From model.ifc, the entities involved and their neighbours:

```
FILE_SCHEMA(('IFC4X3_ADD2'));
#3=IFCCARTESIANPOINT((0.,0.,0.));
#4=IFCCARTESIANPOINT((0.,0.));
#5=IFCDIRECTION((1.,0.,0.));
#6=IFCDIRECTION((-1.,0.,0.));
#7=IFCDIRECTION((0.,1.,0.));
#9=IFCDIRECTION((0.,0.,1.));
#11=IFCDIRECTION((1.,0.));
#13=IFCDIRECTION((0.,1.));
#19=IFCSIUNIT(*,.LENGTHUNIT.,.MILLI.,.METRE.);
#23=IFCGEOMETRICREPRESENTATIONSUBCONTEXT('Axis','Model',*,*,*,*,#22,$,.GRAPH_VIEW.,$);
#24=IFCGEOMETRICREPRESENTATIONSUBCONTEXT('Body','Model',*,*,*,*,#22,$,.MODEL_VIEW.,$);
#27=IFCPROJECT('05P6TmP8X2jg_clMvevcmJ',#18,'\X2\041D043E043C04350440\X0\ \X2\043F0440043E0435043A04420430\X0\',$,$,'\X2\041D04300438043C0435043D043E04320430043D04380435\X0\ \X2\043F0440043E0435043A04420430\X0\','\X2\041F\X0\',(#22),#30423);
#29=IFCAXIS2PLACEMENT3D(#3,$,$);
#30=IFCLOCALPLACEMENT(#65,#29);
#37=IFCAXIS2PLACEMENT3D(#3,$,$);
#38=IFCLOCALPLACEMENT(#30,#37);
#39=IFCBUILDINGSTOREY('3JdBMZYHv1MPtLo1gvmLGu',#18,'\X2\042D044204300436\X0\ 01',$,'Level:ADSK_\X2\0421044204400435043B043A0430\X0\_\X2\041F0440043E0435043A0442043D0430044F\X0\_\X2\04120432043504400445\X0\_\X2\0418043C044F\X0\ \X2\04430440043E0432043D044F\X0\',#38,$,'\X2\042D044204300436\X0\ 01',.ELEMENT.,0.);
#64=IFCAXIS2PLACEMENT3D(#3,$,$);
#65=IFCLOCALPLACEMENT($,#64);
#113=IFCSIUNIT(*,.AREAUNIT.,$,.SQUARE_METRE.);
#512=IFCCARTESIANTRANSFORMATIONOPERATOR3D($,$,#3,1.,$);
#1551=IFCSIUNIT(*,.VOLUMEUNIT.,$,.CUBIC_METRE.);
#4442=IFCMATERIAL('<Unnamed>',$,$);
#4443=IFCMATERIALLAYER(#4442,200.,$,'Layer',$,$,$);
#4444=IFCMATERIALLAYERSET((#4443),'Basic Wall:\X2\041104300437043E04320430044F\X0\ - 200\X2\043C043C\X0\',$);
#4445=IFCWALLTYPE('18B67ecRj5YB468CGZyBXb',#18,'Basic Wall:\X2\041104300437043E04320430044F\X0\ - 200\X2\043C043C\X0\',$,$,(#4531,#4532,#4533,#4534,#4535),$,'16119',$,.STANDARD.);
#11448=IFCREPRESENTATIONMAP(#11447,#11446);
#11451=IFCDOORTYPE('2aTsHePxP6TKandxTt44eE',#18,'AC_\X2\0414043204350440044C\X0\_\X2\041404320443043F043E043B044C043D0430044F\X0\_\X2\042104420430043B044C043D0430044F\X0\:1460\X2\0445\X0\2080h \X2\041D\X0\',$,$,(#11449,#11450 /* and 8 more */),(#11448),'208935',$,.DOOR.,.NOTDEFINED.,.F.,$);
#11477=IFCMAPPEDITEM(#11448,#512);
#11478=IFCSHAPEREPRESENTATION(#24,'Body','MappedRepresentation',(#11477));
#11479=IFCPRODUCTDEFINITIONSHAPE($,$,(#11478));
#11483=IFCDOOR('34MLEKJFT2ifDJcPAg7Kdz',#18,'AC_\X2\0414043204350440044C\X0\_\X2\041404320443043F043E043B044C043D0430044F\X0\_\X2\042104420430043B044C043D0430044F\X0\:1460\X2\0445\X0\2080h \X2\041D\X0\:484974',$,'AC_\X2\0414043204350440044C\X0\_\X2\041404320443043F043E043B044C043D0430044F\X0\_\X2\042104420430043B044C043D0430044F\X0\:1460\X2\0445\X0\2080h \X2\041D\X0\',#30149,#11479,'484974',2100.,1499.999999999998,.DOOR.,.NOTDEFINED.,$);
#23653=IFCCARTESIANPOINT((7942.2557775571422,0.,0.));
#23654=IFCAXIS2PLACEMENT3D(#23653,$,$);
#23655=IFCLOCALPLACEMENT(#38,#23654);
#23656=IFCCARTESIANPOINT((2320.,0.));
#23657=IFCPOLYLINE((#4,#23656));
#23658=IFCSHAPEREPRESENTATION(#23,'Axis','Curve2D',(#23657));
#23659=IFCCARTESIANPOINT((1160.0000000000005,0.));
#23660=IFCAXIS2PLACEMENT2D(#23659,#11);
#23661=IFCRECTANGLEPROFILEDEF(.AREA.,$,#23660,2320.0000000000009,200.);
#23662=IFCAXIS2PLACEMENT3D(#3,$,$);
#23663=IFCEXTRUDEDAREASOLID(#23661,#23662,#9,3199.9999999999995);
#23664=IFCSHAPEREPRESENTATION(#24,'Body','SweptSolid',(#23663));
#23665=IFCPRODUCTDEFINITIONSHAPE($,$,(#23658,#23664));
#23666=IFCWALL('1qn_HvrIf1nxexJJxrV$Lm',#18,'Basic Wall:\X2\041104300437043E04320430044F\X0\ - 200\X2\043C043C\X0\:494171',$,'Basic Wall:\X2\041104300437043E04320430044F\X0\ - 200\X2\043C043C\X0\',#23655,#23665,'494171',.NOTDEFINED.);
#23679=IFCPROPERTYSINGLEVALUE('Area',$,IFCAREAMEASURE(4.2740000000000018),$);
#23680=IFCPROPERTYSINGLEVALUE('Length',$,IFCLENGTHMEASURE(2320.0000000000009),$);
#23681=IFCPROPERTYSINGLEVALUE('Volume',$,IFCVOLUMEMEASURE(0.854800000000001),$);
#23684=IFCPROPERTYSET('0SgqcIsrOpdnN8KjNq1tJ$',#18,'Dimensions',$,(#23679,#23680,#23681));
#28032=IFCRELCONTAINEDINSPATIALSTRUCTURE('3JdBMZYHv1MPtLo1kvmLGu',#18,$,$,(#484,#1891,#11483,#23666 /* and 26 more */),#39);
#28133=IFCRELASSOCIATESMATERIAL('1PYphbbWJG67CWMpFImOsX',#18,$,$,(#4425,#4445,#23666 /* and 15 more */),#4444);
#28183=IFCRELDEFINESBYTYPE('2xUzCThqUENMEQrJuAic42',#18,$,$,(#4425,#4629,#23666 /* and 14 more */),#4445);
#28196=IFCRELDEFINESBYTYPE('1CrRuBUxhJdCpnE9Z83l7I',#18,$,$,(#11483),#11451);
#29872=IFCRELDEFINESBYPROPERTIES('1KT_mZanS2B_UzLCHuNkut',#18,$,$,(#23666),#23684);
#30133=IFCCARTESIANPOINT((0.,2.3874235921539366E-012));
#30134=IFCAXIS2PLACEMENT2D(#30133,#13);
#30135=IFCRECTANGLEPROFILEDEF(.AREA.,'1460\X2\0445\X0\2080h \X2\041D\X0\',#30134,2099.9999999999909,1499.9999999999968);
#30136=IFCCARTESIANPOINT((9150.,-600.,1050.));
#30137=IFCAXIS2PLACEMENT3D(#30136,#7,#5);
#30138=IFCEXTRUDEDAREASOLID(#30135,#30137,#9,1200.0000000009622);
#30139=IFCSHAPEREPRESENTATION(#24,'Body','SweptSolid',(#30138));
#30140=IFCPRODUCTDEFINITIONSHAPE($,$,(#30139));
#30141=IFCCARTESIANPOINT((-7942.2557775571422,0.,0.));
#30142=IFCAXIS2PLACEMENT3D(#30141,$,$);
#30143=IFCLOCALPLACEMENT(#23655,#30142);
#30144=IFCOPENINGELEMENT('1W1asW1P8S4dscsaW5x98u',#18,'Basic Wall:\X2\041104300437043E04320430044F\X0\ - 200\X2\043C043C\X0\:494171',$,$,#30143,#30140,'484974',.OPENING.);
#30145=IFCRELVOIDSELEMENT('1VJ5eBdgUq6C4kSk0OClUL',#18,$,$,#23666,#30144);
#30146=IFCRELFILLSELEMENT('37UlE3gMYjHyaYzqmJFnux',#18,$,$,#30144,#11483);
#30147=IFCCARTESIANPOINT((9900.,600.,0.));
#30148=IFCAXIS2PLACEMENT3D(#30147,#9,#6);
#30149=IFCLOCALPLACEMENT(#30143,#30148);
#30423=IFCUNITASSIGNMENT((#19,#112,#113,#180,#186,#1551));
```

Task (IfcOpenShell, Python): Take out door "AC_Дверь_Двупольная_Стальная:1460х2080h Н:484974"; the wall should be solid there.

```python
import ifcopenshell
import ifcopenshell.api.feature
import ifcopenshell.api.pset
import ifcopenshell.api.root
import ifcopenshell.geom
import ifcopenshell.util.element
import ifcopenshell.util.shape
import ifcopenshell.util.unit

model = ifcopenshell.open("model.ifc")
area_scale = ifcopenshell.util.unit.calculate_unit_scale(model, "AREAUNIT")
volume_scale = ifcopenshell.util.unit.calculate_unit_scale(model, "VOLUMEUNIT")
settings = ifcopenshell.geom.settings()


def volume(element):
    """Net volume in cubic metres, openings subtracted."""
    shape = ifcopenshell.geom.create_shape(settings, element)
    return ifcopenshell.util.shape.get_volume(shape.geometry)


door = model.by_guid("34MLEKJFT2ifDJcPAg7Kdz")
opening = door.FillsVoids[0].RelatingOpeningElement
wall = opening.VoidsElements[0].RelatingBuildingElement
before = volume(wall)

ifcopenshell.api.root.remove_product(model, product=door)
ifcopenshell.api.feature.remove_feature(model, feature=opening)

after = volume(wall)
thickness = 0.2  # wall thickness in metres

# Update the wall's stored quantities.
pset = model.by_id(ifcopenshell.util.element.get_pset(wall, "Dimensions", should_inherit=False)["id"])
ifcopenshell.api.pset.edit_pset(model, pset=pset, properties={
    "Area": model.create_entity("IfcAreaMeasure", after / thickness / area_scale),
    "Volume": model.create_entity("IfcVolumeMeasure", after / volume_scale),
})

print(f"wall volume {before:.3f} -> {after:.3f} m3")

model.write("model_edited.ifc")
```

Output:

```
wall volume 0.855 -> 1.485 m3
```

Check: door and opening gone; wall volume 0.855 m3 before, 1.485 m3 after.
